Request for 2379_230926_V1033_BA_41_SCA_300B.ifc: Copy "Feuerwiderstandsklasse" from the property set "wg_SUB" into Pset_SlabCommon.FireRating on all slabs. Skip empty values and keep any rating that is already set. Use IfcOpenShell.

First a look at what the model holds.

```python
import ifcopenshell
import ifcopenshell.util.element

model = ifcopenshell.open("2379_230926_V1033_BA_41_SCA_300B.ifc")
print(model.schema)
slabs = model.by_type("IfcSlab")
print(len(slabs), "slabs")
for e in slabs[:8]:
    source = ifcopenshell.util.element.get_pset(e, "wg_SUB", "Feuerwiderstandsklasse")
    target = ifcopenshell.util.element.get_pset(e, "Pset_SlabCommon", "FireRating")
    print(e.id(), repr(source), repr(target), sep=" | ")
```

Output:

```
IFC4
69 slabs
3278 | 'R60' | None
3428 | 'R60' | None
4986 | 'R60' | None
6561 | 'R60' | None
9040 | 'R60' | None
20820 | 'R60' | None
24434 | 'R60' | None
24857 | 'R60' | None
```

```python
import ifcopenshell
import ifcopenshell.api.pset
import ifcopenshell.util.element

model = ifcopenshell.open("2379_230926_V1033_BA_41_SCA_300B.ifc")

count = 0
for e in model.by_type("IfcSlab"):
    value = ifcopenshell.util.element.get_pset(e, "wg_SUB", "Feuerwiderstandsklasse")
    current = ifcopenshell.util.element.get_pset(e, "Pset_SlabCommon", "FireRating")
    if not value or not value.strip() or current:
        continue
    # add_pset returns the element's existing set when there is one.
    pset = ifcopenshell.api.pset.add_pset(model, product=e, name="Pset_SlabCommon")
    ifcopenshell.api.pset.edit_pset(model, pset=pset, properties={"FireRating": value})
    count += 1

print(count, "slabs updated")

model.write("2379_230926_V1033_BA_41_SCA_300B_edited.ifc")
```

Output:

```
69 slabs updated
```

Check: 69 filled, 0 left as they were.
